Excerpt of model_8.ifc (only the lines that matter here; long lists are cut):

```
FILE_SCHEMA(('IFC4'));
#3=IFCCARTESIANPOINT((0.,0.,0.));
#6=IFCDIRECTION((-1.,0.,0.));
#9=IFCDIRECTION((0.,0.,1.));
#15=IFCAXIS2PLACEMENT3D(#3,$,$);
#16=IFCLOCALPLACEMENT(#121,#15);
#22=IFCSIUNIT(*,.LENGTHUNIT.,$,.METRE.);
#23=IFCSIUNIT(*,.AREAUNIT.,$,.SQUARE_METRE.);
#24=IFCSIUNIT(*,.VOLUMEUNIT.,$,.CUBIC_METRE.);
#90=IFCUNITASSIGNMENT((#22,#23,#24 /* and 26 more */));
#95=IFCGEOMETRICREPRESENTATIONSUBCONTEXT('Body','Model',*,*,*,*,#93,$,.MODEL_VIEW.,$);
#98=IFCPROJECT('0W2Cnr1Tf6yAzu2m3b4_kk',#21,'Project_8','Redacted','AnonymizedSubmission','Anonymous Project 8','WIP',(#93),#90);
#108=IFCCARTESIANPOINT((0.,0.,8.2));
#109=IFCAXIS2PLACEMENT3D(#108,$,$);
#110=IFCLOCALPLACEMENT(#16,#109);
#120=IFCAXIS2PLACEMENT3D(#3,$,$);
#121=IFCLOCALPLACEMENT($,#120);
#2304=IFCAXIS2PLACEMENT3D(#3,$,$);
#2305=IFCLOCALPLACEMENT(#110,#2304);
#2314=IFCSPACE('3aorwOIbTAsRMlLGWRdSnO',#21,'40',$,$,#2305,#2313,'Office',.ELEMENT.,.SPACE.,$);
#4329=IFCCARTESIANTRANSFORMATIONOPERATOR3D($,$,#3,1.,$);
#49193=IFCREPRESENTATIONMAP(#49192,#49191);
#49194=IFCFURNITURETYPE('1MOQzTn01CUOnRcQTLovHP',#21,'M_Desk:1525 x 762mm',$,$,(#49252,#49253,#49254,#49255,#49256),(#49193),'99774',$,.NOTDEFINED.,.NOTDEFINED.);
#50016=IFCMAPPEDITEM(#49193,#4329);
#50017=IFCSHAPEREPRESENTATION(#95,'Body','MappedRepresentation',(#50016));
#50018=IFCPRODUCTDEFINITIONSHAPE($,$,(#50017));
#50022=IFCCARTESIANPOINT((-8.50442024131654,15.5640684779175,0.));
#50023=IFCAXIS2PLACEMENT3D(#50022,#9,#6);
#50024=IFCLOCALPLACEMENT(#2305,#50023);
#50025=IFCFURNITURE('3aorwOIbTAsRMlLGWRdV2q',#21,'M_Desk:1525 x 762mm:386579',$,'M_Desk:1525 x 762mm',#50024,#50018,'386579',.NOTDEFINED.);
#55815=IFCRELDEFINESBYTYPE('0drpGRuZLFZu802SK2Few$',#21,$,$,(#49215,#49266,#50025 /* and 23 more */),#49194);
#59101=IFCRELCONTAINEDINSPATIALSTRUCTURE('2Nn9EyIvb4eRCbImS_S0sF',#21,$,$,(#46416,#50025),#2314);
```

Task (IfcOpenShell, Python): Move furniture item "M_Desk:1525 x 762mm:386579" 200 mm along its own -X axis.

```python
import ifcopenshell
import ifcopenshell.api.geometry
import ifcopenshell.util.placement

model = ifcopenshell.open("model_8.ifc")

item = model.by_guid("3aorwOIbTAsRMlLGWRdV2q")
matrix = ifcopenshell.util.placement.get_local_placement(item.ObjectPlacement)
matrix[:3, 3] -= matrix[:3, 0] * 0.2
ifcopenshell.api.geometry.edit_object_placement(model, product=item, matrix=matrix, is_si=False)

print(ifcopenshell.util.placement.get_local_placement(item.ObjectPlacement).round(3) + 0.0)

model.write("model_8_rev.ifc")
```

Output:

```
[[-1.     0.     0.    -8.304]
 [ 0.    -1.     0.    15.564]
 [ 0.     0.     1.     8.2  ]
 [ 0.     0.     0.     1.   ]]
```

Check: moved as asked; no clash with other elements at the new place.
